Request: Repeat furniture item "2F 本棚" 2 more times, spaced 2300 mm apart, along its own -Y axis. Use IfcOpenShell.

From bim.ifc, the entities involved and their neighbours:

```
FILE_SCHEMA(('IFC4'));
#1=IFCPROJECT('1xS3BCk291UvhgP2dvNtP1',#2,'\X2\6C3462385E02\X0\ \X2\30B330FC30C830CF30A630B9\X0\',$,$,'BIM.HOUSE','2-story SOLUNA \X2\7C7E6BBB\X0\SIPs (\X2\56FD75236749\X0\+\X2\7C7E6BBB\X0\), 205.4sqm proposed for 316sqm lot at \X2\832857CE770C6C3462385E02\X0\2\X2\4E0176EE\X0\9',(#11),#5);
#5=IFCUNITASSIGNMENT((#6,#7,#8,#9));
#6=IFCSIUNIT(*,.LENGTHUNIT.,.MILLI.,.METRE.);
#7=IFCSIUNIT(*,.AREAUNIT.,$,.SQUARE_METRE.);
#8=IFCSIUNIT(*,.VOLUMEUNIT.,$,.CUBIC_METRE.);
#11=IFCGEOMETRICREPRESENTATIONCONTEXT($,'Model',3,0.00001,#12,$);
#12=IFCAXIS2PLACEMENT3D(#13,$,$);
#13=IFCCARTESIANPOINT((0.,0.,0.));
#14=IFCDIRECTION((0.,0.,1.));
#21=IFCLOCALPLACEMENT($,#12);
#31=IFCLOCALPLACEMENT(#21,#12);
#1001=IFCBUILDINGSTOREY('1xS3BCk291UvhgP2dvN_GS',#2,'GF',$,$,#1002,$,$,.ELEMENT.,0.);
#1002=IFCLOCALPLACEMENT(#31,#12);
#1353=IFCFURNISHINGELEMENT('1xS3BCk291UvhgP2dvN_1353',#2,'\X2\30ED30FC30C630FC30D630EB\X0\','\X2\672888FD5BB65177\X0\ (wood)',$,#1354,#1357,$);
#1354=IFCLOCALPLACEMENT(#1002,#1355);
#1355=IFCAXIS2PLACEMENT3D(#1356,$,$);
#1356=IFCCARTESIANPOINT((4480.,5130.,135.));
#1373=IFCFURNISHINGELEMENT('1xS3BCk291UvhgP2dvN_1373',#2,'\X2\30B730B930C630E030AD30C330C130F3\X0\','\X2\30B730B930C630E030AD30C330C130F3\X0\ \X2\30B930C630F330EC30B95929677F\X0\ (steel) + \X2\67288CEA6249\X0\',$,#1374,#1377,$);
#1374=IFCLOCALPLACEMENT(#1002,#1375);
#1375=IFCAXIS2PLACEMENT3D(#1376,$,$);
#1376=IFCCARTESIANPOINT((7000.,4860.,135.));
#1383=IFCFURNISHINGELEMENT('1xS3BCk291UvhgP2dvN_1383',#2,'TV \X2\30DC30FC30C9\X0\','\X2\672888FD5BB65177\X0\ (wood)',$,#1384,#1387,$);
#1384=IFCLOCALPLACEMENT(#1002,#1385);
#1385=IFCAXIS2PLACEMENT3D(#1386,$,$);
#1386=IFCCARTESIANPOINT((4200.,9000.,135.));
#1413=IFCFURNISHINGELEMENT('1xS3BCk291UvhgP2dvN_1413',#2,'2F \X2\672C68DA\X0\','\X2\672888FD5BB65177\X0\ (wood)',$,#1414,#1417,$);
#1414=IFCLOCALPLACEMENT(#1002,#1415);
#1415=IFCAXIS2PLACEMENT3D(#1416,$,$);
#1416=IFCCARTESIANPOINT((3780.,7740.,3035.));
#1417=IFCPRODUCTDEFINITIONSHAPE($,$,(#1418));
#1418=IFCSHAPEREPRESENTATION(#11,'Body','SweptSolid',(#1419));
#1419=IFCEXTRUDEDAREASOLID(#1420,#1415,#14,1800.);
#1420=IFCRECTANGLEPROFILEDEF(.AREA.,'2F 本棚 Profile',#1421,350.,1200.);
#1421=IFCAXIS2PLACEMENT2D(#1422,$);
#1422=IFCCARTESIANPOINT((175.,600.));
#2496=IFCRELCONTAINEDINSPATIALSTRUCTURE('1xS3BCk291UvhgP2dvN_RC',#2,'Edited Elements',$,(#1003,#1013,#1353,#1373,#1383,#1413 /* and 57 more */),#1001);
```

```python
import ifcopenshell
import ifcopenshell.api.geometry
import ifcopenshell.api.root
import ifcopenshell.util.element
import ifcopenshell.util.placement
import ifcopenshell.util.unit

model = ifcopenshell.open("bim.ifc")
unit_scale = ifcopenshell.util.unit.calculate_unit_scale(model)


def reuse_history(source, copy):
    """copy_class also copies each property set's owner history, people and application; keep the originals."""
    for rel in copy.IsDefinedBy:
        if rel.is_a("IfcRelDefinesByProperties") and (history := rel.RelatingPropertyDefinition.OwnerHistory):
            rel.RelatingPropertyDefinition.OwnerHistory = source.OwnerHistory
            ifcopenshell.util.element.remove_deep2(model, history)


source = model.by_guid("1xS3BCk291UvhgP2dvN_1413")
base = ifcopenshell.util.placement.get_local_placement(source.ObjectPlacement)
step = -base[:3, 1] * 2.3 / unit_scale

for i in range(1, 3):
    copy = ifcopenshell.api.root.copy_class(model, product=source)
    copy.Representation = ifcopenshell.util.element.copy_deep(
        model, source.Representation, exclude=["IfcGeometricRepresentationContext", "IfcRepresentationMap"]
    )
    reuse_history(source, copy)
    matrix = base.copy()
    matrix[:3, 3] += i * step
    print("added at", matrix[:3, 3].round(3) + 0.0)
    ifcopenshell.api.geometry.edit_object_placement(model, product=copy, matrix=matrix, is_si=False)

model.write("bim-out.ifc")
```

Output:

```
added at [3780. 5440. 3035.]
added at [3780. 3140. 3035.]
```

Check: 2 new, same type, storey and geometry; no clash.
